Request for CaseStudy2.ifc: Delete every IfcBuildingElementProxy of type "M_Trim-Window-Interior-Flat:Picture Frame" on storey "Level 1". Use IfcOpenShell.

First a look at what the model holds.

```python
import ifcopenshell
import ifcopenshell.util.element

model = ifcopenshell.open("CaseStudy2.ifc")
print(model.schema)
storey = next(s for s in model.by_type("IfcBuildingStorey") if s.Name == "Level 1")
proxies = [e for e in ifcopenshell.util.element.get_decomposition(storey) if e.is_a("IfcBuildingElementProxy")]
seen = {}
for e in proxies:
    element_type = ifcopenshell.util.element.get_type(e)
    name = element_type.Name if element_type not in (None, e) else None
    seen[name] = seen.get(name, 0) + 1
for name, count in sorted(seen.items(), key=str):
    print(count, "x", name)
```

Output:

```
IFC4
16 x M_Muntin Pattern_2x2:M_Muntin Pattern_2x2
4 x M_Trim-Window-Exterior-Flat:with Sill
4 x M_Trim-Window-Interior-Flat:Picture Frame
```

```python
import ifcopenshell
import ifcopenshell.api.root
import ifcopenshell.util.element

model = ifcopenshell.open("CaseStudy2.ifc")

storey = next(s for s in model.by_type("IfcBuildingStorey") if s.Name == "Level 1")
proxies = [e for e in ifcopenshell.util.element.get_decomposition(storey) if e.is_a("IfcBuildingElementProxy")]
targets = [e for e in proxies if (t := ifcopenshell.util.element.get_type(e)) not in (None, e) and t.Name == "M_Trim-Window-Interior-Flat:Picture Frame"]

for e in targets:
    ifcopenshell.api.root.remove_product(model, product=e)
print(len(targets), "removed")

model.write("CaseStudy2-out.ifc")
```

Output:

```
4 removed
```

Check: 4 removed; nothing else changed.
